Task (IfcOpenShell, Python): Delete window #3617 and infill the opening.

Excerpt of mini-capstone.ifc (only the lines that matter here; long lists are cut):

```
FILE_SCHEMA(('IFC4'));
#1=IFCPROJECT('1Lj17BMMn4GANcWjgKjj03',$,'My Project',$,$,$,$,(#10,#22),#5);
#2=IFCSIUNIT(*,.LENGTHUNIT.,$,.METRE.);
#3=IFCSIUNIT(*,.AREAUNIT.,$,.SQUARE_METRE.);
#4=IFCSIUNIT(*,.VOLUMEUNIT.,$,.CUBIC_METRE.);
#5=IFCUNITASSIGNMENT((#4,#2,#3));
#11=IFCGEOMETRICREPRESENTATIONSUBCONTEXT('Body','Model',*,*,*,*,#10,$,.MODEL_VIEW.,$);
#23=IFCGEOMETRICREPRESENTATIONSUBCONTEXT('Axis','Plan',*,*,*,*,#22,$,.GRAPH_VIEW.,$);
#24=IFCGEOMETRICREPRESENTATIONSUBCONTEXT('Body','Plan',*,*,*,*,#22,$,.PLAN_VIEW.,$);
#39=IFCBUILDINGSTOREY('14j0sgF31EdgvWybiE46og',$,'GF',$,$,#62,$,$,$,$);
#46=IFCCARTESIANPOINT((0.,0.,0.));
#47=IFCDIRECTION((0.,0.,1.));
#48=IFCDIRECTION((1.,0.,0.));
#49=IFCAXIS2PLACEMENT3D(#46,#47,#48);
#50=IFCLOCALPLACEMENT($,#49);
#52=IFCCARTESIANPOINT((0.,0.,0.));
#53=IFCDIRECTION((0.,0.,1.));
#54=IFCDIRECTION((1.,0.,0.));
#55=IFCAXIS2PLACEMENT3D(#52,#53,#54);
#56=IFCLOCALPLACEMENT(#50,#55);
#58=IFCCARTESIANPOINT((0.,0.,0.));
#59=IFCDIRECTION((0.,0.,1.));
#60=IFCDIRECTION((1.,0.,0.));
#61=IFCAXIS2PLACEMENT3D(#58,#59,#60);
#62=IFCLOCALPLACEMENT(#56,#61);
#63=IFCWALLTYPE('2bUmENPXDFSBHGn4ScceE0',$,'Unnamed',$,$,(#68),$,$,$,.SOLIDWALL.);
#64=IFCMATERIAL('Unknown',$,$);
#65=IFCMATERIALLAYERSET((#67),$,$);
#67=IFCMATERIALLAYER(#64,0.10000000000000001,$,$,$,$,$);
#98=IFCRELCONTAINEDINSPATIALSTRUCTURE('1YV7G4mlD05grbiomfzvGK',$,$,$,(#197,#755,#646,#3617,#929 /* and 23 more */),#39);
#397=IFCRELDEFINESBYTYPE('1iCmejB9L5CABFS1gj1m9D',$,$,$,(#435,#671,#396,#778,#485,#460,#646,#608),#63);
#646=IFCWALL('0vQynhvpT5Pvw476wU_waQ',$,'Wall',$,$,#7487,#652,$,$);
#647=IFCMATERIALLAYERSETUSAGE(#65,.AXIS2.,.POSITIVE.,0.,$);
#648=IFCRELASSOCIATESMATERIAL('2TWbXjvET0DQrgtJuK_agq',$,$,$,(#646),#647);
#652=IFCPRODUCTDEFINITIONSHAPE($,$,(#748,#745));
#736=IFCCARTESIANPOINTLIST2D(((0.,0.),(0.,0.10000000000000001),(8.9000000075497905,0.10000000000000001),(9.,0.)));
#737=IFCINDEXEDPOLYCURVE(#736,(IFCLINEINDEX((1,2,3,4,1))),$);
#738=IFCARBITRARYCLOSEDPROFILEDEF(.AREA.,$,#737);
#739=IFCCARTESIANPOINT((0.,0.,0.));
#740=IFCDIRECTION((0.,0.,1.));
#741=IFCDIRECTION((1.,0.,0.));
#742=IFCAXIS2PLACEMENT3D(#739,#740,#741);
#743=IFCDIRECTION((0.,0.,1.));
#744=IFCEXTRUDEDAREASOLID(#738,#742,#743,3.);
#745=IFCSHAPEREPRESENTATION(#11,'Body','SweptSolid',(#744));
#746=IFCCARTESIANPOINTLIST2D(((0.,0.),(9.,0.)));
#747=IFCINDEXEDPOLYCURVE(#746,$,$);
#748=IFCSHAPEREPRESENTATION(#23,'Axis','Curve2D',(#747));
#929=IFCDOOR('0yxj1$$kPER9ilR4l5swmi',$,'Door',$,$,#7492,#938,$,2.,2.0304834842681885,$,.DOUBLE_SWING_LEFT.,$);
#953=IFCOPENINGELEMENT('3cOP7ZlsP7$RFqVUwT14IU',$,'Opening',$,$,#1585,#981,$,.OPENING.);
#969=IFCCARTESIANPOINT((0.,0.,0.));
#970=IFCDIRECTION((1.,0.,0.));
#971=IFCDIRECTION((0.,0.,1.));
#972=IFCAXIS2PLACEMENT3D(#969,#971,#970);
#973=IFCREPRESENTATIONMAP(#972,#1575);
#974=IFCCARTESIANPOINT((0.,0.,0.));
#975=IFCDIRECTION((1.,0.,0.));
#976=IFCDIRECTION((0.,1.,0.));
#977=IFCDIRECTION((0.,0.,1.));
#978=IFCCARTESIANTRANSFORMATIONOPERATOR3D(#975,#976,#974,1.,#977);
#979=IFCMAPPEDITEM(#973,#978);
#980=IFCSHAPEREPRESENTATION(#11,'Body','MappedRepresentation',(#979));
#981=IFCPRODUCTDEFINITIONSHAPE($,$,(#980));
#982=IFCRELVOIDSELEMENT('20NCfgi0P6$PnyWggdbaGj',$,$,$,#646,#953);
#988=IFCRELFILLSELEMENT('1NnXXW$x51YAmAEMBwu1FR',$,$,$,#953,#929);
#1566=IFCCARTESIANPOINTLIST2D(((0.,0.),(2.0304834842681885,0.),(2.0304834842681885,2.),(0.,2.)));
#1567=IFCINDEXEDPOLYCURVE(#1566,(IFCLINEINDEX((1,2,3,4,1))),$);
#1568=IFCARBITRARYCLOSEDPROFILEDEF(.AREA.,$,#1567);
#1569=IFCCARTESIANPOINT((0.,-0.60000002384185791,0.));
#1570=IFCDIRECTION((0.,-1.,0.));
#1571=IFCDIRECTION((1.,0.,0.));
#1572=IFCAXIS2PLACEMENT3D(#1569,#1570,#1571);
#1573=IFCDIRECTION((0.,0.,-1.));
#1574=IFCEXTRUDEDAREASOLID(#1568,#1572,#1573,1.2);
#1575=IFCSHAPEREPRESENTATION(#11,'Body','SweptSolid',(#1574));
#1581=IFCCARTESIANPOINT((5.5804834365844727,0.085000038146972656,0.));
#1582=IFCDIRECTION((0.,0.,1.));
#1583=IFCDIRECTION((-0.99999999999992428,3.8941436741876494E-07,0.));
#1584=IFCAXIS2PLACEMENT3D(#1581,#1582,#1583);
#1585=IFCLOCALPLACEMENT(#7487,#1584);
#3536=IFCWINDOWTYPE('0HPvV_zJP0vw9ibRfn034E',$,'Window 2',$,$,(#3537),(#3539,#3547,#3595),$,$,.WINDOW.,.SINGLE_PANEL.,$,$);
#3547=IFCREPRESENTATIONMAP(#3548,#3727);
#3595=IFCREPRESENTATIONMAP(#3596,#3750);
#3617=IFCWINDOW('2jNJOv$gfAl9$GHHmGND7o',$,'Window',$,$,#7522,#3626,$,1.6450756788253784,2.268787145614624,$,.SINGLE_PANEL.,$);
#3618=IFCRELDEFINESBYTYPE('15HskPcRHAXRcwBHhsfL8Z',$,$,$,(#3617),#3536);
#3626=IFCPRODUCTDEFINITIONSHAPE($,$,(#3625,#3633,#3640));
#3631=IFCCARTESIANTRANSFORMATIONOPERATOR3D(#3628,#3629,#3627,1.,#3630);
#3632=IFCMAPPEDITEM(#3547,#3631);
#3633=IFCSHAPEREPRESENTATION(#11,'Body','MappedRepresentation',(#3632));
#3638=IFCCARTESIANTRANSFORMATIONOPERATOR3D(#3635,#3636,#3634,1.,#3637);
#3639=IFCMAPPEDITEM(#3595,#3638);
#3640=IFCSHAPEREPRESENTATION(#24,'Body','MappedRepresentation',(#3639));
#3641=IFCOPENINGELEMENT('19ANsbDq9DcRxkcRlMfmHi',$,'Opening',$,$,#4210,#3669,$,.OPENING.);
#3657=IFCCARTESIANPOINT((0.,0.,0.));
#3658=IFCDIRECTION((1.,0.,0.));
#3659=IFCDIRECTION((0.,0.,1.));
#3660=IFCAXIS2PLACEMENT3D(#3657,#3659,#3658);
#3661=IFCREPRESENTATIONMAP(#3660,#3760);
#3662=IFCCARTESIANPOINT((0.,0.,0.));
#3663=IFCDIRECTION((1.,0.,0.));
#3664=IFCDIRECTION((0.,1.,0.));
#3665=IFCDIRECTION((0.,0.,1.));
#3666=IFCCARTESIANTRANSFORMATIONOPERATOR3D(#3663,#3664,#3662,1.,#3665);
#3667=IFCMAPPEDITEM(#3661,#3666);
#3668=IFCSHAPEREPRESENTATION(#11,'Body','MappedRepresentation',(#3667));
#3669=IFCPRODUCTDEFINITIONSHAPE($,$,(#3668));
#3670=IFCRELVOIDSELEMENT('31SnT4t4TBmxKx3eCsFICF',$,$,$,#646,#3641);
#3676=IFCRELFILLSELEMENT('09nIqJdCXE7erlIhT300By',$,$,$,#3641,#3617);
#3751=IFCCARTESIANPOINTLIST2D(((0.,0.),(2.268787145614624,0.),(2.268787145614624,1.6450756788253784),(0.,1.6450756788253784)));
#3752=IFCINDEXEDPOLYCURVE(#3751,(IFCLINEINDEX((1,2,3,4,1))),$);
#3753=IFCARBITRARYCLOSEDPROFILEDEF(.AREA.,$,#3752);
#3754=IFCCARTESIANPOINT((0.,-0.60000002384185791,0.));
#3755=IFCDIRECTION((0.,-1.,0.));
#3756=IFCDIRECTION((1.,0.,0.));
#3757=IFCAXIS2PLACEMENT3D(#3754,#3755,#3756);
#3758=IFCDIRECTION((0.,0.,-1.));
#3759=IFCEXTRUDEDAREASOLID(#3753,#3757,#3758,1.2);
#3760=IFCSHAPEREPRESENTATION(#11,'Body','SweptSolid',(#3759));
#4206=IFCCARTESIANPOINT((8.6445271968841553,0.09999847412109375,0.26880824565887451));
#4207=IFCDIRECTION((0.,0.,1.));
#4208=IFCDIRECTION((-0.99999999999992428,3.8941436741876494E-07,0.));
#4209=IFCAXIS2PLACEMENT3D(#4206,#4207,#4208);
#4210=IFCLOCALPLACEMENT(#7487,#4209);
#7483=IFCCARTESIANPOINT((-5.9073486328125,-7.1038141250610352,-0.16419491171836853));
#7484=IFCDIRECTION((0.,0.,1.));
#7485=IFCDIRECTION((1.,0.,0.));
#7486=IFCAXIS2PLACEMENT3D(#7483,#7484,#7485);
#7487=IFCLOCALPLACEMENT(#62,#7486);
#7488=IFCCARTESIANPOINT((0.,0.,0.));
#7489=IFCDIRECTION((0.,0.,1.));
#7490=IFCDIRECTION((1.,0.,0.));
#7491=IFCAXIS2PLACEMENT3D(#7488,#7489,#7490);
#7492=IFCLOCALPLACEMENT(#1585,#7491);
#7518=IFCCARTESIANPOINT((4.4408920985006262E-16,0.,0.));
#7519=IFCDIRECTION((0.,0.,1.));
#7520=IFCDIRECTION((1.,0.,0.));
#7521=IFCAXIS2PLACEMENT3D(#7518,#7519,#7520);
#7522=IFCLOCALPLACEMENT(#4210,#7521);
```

```python
import ifcopenshell
import ifcopenshell.api.feature
import ifcopenshell.api.root
import ifcopenshell.geom
import ifcopenshell.util.shape

model = ifcopenshell.open("mini-capstone.ifc")
settings = ifcopenshell.geom.settings()


def volume(element):
    """Net volume in cubic metres, openings subtracted."""
    shape = ifcopenshell.geom.create_shape(settings, element)
    return ifcopenshell.util.shape.get_volume(shape.geometry)


window = model.by_id(3617)
opening = window.FillsVoids[0].RelatingOpeningElement
wall = opening.VoidsElements[0].RelatingBuildingElement
before = volume(wall)

ifcopenshell.api.root.remove_product(model, product=window)
ifcopenshell.api.feature.remove_feature(model, feature=opening)

after = volume(wall)

print(f"wall volume {before:.3f} -> {after:.3f} m3")

model.write("mini-capstone_v2.ifc")
```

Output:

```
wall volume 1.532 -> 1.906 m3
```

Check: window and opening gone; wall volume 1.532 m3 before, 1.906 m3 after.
